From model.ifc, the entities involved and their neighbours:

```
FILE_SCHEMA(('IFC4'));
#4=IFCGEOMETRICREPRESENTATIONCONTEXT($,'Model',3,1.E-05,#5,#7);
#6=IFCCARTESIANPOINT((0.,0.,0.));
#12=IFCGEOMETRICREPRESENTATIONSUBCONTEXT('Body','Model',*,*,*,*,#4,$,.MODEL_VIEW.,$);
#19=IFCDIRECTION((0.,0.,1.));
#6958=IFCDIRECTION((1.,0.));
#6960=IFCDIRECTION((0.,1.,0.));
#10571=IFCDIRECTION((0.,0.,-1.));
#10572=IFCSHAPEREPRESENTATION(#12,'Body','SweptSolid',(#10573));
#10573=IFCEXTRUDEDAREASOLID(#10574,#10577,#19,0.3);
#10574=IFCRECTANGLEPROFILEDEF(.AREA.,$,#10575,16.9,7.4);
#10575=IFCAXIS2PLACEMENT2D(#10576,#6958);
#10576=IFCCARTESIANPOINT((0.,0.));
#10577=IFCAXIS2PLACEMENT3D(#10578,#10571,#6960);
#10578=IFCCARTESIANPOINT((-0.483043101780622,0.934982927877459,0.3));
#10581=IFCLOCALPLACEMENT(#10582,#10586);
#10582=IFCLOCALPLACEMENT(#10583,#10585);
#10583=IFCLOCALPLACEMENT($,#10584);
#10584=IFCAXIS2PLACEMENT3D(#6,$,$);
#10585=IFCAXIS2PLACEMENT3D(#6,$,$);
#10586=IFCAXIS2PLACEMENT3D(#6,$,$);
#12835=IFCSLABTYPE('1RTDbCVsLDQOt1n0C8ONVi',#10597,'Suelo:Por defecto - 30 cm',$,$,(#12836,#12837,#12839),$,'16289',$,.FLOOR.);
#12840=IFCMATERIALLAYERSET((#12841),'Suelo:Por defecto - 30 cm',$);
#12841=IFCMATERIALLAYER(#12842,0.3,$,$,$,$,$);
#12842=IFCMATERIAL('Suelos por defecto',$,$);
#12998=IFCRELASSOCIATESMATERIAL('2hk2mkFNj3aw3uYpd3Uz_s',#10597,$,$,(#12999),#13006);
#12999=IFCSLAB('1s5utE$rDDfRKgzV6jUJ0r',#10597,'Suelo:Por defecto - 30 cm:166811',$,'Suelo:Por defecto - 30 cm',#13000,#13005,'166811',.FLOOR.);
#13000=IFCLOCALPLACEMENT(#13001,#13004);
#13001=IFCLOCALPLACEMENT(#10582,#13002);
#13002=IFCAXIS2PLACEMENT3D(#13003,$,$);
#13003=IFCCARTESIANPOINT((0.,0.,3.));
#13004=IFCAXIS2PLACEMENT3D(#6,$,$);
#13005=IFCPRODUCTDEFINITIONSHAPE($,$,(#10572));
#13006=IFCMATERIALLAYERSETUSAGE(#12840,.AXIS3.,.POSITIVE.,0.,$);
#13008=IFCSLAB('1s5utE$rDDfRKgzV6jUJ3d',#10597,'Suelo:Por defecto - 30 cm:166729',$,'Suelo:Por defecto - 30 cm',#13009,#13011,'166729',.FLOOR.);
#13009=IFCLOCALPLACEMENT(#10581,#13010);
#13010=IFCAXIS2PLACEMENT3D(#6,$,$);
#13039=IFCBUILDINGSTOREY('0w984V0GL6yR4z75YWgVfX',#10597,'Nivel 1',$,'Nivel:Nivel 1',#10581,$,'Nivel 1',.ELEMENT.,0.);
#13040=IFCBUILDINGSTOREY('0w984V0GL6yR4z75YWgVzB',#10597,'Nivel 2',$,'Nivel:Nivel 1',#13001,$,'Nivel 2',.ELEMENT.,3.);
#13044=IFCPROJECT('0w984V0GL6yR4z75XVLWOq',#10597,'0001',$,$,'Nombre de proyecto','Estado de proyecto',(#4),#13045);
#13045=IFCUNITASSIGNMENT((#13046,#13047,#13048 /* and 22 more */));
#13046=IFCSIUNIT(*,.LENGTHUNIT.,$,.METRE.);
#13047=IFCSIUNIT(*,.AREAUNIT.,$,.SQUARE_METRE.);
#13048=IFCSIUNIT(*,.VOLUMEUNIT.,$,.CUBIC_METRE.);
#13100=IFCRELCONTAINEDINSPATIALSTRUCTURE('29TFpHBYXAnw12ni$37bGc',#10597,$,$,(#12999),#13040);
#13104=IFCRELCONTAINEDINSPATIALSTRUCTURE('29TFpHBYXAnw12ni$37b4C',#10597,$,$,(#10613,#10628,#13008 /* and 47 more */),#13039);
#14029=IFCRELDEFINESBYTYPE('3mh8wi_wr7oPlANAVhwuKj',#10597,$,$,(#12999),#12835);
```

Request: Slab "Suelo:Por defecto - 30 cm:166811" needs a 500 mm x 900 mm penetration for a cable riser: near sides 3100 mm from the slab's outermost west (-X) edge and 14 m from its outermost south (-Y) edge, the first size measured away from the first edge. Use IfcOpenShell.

```python
import numpy as np
import ifcopenshell
import ifcopenshell.api.feature
import ifcopenshell.api.geometry
import ifcopenshell.api.root
import ifcopenshell.geom
import ifcopenshell.util.placement
import ifcopenshell.util.representation
import ifcopenshell.util.shape
import ifcopenshell.util.unit

model = ifcopenshell.open("model.ifc")
unit_scale = ifcopenshell.util.unit.calculate_unit_scale(model)
settings = ifcopenshell.geom.settings()


def volume(element):
    """Net volume in cubic metres, openings subtracted."""
    shape = ifcopenshell.geom.create_shape(settings, element)
    return ifcopenshell.util.shape.get_volume(shape.geometry)


slab = model.by_id(12999)
before = volume(slab)

# Extent in the slab's own axes, in metres. The edges named are its -X and -Y sides.
slab_shape = ifcopenshell.geom.create_shape(settings, slab)
vertices = ifcopenshell.util.shape.get_vertices(slab_shape.geometry)
x_min, y_min, bottom = vertices.min(axis=0)
top = vertices[:, 2].max()

opening = ifcopenshell.api.root.create_entity(model, ifc_class="IfcOpeningElement", name="Cable riser opening", predefined_type="OPENING")
context = ifcopenshell.util.representation.get_context(model, "Model", "Body", "MODEL_VIEW")
width, depth = 0.5, 0.9
outline = [(0.0, 0.0), (width, 0.0), (width, depth), (0.0, depth), (0.0, 0.0)]
# Overshoot both faces by 50 mm so the cut is clean.
shape = ifcopenshell.api.geometry.add_slab_representation(
    model, context=context, depth=top - bottom + 0.1, polyline=outline
)
ifcopenshell.api.geometry.assign_representation(model, product=opening, representation=shape)

matrix = ifcopenshell.util.placement.get_local_placement(slab.ObjectPlacement)
matrix[:, 3] = matrix @ np.append(np.array([x_min + 3.1, y_min + 14, bottom - 0.05]) / unit_scale, 1.0)
ifcopenshell.api.geometry.edit_object_placement(model, product=opening, matrix=matrix, is_si=False)
ifcopenshell.api.feature.add_feature(model, feature=opening, element=slab)

after = volume(slab)

print(f"slab volume {before:.3f} -> {after:.3f} m3")

model.write("model-out.ifc")
```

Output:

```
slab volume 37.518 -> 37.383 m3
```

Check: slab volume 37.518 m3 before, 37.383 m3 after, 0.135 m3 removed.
